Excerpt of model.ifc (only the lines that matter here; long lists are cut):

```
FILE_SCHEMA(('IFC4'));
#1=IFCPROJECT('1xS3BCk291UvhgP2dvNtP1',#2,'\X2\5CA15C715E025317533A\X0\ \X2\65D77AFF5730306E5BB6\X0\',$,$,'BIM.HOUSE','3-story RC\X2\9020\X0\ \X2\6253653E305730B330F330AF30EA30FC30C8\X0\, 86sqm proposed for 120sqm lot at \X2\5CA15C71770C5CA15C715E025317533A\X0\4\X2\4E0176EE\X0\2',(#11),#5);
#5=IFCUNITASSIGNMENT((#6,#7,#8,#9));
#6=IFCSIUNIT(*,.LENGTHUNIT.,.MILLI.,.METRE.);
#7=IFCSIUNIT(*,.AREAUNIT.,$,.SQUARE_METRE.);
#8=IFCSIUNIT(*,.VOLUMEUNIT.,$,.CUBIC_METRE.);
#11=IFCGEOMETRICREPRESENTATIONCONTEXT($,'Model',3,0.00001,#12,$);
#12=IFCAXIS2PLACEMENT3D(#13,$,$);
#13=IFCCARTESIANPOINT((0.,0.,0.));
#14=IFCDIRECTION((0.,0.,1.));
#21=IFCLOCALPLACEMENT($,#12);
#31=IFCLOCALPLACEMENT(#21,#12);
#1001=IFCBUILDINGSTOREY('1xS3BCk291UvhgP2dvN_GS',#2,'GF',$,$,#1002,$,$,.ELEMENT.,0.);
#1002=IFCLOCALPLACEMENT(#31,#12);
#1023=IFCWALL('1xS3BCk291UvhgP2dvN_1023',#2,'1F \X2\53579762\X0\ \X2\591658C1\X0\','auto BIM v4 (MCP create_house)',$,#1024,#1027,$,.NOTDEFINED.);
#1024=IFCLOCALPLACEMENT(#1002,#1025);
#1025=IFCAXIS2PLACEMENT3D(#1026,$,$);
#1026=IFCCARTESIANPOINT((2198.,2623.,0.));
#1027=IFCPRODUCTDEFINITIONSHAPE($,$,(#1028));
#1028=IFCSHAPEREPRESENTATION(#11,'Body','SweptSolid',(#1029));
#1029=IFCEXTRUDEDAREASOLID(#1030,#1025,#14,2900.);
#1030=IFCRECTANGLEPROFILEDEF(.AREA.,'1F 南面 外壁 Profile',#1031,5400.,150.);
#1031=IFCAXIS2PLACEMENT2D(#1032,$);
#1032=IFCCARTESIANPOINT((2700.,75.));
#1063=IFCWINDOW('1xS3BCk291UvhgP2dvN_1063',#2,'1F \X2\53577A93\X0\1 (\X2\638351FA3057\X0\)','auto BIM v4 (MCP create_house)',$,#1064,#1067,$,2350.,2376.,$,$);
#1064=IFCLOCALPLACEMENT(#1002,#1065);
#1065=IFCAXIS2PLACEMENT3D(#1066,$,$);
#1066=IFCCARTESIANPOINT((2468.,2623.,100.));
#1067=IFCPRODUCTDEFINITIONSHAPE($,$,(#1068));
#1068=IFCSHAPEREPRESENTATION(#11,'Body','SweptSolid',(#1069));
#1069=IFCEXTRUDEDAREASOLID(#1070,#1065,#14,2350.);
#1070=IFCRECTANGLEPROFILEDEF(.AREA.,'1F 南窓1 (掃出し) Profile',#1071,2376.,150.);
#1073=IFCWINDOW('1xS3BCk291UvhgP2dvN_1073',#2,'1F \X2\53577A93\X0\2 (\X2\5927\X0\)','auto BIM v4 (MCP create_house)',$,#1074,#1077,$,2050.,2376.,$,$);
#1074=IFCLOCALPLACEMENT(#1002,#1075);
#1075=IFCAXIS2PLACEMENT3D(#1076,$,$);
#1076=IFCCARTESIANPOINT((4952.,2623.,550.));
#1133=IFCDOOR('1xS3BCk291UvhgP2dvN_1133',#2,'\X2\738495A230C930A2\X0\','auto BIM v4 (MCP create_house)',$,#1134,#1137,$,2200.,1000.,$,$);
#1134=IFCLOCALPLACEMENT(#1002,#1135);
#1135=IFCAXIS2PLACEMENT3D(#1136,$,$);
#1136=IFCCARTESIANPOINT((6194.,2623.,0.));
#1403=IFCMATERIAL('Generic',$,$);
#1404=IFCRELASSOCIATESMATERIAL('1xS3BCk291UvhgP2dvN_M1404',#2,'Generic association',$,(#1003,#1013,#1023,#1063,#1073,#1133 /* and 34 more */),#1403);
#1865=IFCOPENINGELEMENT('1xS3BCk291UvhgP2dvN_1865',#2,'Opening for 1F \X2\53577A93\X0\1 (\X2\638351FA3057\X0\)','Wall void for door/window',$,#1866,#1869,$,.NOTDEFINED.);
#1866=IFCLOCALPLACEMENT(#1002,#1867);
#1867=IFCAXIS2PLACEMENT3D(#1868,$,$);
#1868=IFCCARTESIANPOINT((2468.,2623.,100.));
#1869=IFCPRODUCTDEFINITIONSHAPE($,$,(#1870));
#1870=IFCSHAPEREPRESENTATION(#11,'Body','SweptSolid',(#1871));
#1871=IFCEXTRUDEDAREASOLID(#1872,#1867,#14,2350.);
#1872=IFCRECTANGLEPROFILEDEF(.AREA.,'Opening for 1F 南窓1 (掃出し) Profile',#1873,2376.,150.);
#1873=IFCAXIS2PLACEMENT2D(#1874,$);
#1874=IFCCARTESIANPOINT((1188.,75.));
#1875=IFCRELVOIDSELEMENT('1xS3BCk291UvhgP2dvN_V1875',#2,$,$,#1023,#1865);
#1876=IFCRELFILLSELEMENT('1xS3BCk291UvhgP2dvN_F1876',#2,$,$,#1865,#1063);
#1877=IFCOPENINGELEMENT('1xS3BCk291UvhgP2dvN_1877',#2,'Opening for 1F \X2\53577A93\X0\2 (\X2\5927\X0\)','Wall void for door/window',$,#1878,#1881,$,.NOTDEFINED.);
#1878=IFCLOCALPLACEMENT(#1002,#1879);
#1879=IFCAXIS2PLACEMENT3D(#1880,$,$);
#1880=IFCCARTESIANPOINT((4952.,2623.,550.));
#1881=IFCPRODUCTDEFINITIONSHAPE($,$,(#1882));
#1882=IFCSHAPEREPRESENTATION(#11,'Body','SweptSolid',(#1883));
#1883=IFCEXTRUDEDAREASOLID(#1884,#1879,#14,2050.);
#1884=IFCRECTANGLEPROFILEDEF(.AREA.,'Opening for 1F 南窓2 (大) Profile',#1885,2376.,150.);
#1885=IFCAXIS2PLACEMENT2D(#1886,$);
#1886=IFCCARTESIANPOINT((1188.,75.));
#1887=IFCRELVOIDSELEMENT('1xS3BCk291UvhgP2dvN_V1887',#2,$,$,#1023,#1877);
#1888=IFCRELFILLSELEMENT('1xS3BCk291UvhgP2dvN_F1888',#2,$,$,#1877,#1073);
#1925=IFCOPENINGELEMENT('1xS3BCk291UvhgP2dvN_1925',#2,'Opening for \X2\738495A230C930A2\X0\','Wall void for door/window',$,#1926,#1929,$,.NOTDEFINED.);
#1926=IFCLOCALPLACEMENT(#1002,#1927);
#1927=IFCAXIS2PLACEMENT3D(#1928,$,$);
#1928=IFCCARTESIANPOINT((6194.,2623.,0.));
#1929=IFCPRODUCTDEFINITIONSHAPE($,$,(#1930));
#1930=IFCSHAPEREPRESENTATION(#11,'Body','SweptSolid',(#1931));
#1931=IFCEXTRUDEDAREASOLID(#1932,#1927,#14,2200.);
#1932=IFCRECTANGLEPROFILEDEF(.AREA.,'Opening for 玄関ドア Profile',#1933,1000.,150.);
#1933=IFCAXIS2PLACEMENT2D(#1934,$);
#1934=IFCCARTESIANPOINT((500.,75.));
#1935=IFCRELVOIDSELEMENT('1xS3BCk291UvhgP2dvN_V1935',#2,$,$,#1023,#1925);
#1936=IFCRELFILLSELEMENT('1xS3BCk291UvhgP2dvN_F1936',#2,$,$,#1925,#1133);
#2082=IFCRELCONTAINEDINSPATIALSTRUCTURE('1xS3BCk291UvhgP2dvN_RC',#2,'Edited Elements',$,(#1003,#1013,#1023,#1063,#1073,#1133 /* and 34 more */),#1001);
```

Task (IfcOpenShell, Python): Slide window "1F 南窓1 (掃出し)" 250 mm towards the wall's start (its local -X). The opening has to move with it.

```python
import ifcopenshell
import ifcopenshell.api.geometry
import ifcopenshell.util.placement

model = ifcopenshell.open("model.ifc")

window = model.by_guid("1xS3BCk291UvhgP2dvN_1063")
opening = window.FillsVoids[0].RelatingOpeningElement
wall = opening.VoidsElements[0].RelatingBuildingElement

wall_matrix = ifcopenshell.util.placement.get_local_placement(wall.ObjectPlacement)
shift = wall_matrix[:3, 0] * -250.0
before = ifcopenshell.util.placement.get_local_placement(window.ObjectPlacement)[:3, 3].copy()

# The window is not placed relative to its opening, so move both.
for product in (opening, window):
    matrix = ifcopenshell.util.placement.get_local_placement(product.ObjectPlacement)
    matrix[:3, 3] += shift
    ifcopenshell.api.geometry.edit_object_placement(model, product=product, matrix=matrix, is_si=False)

after = ifcopenshell.util.placement.get_local_placement(window.ObjectPlacement)[:3, 3]
print("window moved by", (after - before).round(3) + 0.0)

model.write("model_edited.ifc")
```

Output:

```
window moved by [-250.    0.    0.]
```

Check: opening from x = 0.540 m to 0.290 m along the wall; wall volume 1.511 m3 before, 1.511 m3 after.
